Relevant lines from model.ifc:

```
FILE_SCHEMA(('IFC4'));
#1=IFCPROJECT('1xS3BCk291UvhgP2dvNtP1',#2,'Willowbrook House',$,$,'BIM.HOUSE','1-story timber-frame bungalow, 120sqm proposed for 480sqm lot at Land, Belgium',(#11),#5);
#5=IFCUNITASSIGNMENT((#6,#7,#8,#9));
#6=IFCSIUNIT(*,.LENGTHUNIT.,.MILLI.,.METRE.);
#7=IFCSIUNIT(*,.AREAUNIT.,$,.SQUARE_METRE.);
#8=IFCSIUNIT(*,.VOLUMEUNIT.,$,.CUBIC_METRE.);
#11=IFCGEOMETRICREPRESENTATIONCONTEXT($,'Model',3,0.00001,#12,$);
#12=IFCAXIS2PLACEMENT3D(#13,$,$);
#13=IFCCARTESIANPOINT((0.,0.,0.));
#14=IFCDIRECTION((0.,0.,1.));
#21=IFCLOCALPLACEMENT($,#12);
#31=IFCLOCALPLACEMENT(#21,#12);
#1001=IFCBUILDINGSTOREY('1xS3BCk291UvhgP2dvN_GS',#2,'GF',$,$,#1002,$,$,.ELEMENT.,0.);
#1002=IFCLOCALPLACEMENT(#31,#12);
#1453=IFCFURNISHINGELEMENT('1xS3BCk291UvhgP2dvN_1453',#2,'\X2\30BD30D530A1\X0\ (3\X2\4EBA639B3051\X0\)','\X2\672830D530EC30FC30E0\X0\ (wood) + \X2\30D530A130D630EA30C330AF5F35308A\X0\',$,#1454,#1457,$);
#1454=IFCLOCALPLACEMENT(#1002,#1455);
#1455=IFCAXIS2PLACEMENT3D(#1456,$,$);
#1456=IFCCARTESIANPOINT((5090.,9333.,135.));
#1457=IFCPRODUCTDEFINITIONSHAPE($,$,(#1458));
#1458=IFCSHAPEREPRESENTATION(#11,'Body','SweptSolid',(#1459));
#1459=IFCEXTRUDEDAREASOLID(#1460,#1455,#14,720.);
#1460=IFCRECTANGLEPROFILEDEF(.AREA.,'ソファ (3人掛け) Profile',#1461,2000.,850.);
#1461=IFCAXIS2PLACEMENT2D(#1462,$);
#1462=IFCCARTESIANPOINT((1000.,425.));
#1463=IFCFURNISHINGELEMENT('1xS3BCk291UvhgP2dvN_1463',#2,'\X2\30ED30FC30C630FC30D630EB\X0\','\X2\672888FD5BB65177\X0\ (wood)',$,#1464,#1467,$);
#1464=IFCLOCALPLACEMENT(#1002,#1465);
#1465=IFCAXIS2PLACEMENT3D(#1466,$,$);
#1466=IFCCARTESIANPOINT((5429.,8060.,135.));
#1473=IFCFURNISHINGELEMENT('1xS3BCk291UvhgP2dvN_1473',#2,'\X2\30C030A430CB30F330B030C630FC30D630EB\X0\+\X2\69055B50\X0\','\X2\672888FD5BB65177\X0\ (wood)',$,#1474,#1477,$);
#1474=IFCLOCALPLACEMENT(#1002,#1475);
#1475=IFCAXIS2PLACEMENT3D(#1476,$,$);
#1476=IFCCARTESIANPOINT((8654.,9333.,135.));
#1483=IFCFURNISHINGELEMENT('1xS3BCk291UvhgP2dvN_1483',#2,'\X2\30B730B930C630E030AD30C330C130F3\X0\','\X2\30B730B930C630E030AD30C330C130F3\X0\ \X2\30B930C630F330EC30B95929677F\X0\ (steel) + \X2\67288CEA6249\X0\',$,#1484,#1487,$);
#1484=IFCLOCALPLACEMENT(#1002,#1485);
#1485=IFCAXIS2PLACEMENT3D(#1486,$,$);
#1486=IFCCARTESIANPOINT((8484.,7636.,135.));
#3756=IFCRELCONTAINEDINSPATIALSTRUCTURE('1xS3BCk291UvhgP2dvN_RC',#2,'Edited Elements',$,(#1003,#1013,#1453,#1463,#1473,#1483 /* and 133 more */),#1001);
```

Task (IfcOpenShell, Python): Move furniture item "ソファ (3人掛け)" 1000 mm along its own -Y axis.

```python
import ifcopenshell
import ifcopenshell.api.geometry
import ifcopenshell.util.placement

model = ifcopenshell.open("model.ifc")

item = model.by_guid("1xS3BCk291UvhgP2dvN_1453")
matrix = ifcopenshell.util.placement.get_local_placement(item.ObjectPlacement)
matrix[:3, 3] -= matrix[:3, 1] * 1000.0
ifcopenshell.api.geometry.edit_object_placement(model, product=item, matrix=matrix, is_si=False)

print(ifcopenshell.util.placement.get_local_placement(item.ObjectPlacement).round(3) + 0.0)

model.write("model_edited.ifc")
```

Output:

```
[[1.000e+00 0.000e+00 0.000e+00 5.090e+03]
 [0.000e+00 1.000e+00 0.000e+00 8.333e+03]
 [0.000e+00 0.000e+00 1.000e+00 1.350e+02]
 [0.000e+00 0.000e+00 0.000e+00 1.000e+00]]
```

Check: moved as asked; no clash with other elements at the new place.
